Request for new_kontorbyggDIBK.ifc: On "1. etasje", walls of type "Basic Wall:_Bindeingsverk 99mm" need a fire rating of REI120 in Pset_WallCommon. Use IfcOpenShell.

First a look at what the model holds.

```python
import ifcopenshell
import ifcopenshell.util.element

model = ifcopenshell.open("new_kontorbyggDIBK.ifc")
print(model.schema)
storey = next(s for s in model.by_type("IfcBuildingStorey") if s.Name == "1. etasje")
walls = [e for e in ifcopenshell.util.element.get_decomposition(storey) if e.is_a("IfcWall")]
seen = {}
for e in walls:
    element_type = ifcopenshell.util.element.get_type(e)
    key = (element_type.Name if element_type != e and element_type else None, ifcopenshell.util.element.get_pset(e, "Pset_WallCommon", "FireRating"))
    seen[key] = seen.get(key, 0) + 1
for (name, value), count in sorted(seen.items(), key=str):
    print(count, "x", name, "|", value)
```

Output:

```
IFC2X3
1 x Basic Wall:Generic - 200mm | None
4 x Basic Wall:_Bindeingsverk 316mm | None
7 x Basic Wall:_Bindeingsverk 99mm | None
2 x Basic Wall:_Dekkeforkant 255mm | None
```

```python
import ifcopenshell
import ifcopenshell.api.pset
import ifcopenshell.util.element

model = ifcopenshell.open("new_kontorbyggDIBK.ifc")

storey = next(s for s in model.by_type("IfcBuildingStorey") if s.Name == "1. etasje")
walls = [e for e in ifcopenshell.util.element.get_decomposition(storey) if e.is_a("IfcWall")]

count = 0
for e in walls:
    element_type = ifcopenshell.util.element.get_type(e)
    if element_type in (None, e) or element_type.Name != "Basic Wall:_Bindeingsverk 99mm":
        continue
    # add_pset returns the element's existing set when there is one.
    pset = ifcopenshell.api.pset.add_pset(model, product=e, name="Pset_WallCommon")
    ifcopenshell.api.pset.edit_pset(model, pset=pset, properties={"FireRating": "REI120"})
    count += 1

print(count, "walls updated")

model.write("new_kontorbyggDIBK_rev.ifc")
```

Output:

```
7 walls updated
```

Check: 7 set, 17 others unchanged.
